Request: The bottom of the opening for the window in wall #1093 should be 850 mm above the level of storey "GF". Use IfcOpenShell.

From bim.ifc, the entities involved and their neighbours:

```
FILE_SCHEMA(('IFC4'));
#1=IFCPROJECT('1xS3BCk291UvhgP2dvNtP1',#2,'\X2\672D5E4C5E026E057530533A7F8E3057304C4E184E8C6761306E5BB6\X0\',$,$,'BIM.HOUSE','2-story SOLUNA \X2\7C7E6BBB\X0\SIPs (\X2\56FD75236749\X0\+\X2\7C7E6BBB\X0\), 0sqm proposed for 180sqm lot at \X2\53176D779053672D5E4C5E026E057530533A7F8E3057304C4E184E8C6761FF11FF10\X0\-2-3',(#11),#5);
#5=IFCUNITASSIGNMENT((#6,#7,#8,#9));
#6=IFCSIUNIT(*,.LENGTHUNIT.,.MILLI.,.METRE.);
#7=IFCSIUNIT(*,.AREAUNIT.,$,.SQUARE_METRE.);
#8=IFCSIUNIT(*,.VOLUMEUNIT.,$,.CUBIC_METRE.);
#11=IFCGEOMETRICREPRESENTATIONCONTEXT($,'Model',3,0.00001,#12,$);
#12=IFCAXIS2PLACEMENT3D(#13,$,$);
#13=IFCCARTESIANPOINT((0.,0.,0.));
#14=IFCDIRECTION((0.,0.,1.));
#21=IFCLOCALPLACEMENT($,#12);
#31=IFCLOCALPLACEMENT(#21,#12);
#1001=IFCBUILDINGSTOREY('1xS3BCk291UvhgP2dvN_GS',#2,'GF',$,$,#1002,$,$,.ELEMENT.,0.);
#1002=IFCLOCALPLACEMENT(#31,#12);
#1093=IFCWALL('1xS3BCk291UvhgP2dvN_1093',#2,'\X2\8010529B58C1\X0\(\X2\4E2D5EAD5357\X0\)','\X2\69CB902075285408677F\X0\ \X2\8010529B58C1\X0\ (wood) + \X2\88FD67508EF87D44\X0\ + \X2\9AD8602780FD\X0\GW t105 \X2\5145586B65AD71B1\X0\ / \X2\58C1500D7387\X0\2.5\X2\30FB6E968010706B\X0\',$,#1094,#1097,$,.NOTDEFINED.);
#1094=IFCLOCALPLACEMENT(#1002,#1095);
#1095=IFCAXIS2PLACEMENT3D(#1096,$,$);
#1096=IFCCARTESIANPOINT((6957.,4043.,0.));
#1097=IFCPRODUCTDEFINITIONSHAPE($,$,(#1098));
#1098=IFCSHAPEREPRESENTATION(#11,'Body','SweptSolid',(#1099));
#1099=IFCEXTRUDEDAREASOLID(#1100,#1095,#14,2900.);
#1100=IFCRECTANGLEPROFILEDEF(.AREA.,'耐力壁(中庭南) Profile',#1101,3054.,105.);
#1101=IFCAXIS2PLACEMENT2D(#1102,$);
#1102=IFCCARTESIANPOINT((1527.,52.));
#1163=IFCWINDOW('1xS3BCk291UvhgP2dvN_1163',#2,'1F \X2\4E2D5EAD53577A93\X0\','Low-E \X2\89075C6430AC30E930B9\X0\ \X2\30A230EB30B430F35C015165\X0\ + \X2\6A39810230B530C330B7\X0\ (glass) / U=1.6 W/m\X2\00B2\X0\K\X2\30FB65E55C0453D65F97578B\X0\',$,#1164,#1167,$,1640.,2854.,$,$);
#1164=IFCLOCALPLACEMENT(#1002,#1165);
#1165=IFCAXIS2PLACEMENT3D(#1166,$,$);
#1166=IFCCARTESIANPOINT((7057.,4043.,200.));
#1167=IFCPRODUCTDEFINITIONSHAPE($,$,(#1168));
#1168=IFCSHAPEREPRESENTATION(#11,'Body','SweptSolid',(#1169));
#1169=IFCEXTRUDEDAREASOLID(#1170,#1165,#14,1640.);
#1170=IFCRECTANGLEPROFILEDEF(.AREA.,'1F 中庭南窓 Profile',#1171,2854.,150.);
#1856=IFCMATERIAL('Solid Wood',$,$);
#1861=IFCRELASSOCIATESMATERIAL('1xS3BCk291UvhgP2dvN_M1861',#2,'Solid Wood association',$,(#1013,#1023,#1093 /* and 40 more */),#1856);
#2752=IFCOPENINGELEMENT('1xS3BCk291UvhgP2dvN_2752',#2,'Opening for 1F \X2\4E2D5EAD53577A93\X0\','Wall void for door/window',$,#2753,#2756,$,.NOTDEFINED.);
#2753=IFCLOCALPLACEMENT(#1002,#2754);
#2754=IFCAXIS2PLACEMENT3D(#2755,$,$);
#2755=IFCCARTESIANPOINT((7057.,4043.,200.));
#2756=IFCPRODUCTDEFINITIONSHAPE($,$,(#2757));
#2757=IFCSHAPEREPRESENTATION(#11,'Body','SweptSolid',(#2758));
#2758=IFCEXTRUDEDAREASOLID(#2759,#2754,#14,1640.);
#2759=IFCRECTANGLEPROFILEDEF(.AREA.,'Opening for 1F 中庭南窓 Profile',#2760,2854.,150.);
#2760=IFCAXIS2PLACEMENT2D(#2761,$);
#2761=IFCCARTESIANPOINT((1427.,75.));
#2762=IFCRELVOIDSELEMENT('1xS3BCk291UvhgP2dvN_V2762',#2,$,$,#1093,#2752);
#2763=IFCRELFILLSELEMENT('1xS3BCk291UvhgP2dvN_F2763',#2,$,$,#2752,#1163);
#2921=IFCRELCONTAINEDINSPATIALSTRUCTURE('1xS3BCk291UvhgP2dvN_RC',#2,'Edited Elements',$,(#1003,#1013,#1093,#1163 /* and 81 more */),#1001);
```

```python
import numpy as np
import ifcopenshell
import ifcopenshell.api.geometry
import ifcopenshell.geom
import ifcopenshell.util.element
import ifcopenshell.util.placement
import ifcopenshell.util.shape
import ifcopenshell.util.unit

model = ifcopenshell.open("bim.ifc")
unit_scale = ifcopenshell.util.unit.calculate_unit_scale(model)

window = model.by_guid("1xS3BCk291UvhgP2dvN_1163")
opening = window.FillsVoids[0].RelatingOpeningElement
storey = ifcopenshell.util.element.get_container(window, ifc_class="IfcBuildingStorey")
level = ifcopenshell.util.placement.get_local_placement(storey.ObjectPlacement)[2, 3]

# The opening's origin need not be at the sill, so measure its lowest point.
shape = ifcopenshell.geom.create_shape(ifcopenshell.geom.settings(), opening)
bottom = ifcopenshell.util.shape.get_shape_bottom_elevation(shape, shape.geometry) / unit_scale
dz = level + 850.0 - bottom

shift = np.array([0.0, 0.0, dz])
# The window is not placed relative to its opening, so move both.
for product in (opening, window):
    matrix = ifcopenshell.util.placement.get_local_placement(product.ObjectPlacement)
    matrix[:3, 3] += shift
    ifcopenshell.api.geometry.edit_object_placement(model, product=product, matrix=matrix, is_si=False)

print(f"moved by {dz * unit_scale:+.3f} m")

model.write("bim_v2.ifc")
```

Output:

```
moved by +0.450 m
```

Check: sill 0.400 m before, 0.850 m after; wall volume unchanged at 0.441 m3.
